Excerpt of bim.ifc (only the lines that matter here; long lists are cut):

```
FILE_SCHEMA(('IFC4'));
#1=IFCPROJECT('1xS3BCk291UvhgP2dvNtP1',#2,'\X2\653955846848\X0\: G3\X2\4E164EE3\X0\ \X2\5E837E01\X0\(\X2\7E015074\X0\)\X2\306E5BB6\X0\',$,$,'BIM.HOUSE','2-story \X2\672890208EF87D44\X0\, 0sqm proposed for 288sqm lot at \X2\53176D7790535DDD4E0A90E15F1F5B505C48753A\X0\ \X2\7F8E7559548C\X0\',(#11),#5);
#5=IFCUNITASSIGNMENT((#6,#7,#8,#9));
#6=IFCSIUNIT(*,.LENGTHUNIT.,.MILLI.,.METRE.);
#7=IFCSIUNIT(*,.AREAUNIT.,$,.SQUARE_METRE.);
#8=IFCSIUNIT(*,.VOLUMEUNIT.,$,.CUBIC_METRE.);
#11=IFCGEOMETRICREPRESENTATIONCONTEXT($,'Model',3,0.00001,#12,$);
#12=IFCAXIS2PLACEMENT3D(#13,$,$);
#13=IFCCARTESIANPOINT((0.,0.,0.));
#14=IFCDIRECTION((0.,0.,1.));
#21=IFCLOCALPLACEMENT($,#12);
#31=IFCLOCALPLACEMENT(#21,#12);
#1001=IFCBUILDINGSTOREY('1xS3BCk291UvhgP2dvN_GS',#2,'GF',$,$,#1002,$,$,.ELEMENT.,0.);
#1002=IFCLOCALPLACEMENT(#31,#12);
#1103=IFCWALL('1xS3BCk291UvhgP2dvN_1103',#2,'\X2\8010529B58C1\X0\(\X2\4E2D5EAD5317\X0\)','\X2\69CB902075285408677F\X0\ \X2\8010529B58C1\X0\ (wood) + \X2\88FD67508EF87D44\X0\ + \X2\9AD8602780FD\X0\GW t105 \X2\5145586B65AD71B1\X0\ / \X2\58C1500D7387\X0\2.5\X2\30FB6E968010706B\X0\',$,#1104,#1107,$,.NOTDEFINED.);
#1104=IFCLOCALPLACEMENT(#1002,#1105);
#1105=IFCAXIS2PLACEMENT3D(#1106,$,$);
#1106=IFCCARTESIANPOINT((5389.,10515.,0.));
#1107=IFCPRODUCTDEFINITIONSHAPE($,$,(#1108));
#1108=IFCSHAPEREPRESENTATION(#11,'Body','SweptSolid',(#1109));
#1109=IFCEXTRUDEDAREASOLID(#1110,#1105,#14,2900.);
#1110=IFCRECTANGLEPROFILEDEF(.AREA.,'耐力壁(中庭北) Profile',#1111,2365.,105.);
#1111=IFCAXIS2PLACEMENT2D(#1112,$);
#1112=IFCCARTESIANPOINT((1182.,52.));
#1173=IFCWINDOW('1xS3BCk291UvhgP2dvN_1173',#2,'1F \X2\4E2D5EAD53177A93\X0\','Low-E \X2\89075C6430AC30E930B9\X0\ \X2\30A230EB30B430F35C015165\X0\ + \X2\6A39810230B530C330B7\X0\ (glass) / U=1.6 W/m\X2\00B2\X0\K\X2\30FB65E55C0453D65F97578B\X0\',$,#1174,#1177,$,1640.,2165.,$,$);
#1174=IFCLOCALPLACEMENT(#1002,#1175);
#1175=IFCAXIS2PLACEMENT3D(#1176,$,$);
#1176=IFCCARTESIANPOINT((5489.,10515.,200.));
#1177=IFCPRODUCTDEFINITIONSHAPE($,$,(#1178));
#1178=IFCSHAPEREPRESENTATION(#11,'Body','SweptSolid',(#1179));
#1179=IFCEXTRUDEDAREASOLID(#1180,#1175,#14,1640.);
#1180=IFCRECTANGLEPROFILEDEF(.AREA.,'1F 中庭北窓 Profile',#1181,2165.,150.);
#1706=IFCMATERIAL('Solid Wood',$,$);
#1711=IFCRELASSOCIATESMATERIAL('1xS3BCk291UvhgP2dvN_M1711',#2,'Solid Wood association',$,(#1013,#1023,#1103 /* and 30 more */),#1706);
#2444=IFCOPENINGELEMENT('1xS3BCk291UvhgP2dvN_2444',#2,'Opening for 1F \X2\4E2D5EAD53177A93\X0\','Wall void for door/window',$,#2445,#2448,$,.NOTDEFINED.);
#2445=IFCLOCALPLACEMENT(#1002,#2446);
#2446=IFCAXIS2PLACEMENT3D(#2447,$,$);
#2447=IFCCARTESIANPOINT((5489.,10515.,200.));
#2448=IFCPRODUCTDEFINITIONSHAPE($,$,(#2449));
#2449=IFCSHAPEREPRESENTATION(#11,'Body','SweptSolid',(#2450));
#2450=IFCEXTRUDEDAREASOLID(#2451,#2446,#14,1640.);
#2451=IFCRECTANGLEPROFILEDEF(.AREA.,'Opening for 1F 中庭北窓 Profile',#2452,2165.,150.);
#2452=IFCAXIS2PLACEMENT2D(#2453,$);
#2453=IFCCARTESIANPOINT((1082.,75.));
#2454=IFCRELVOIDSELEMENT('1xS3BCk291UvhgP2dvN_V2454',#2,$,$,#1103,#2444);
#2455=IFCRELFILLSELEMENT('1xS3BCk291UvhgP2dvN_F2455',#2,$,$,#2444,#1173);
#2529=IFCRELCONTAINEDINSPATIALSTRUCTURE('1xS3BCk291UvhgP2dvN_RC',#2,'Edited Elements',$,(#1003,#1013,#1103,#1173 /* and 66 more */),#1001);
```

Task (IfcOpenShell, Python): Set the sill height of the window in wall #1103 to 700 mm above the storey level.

```python
import numpy as np
import ifcopenshell
import ifcopenshell.api.geometry
import ifcopenshell.geom
import ifcopenshell.util.element
import ifcopenshell.util.placement
import ifcopenshell.util.shape
import ifcopenshell.util.unit

model = ifcopenshell.open("bim.ifc")
unit_scale = ifcopenshell.util.unit.calculate_unit_scale(model)

window = model.by_guid("1xS3BCk291UvhgP2dvN_1173")
opening = window.FillsVoids[0].RelatingOpeningElement
storey = ifcopenshell.util.element.get_container(window, ifc_class="IfcBuildingStorey")
level = ifcopenshell.util.placement.get_local_placement(storey.ObjectPlacement)[2, 3]

# The opening's origin need not be at the sill, so measure its lowest point.
shape = ifcopenshell.geom.create_shape(ifcopenshell.geom.settings(), opening)
bottom = ifcopenshell.util.shape.get_shape_bottom_elevation(shape, shape.geometry) / unit_scale
dz = level + 700.0 - bottom

shift = np.array([0.0, 0.0, dz])
# The window is not placed relative to its opening, so move both.
for product in (opening, window):
    matrix = ifcopenshell.util.placement.get_local_placement(product.ObjectPlacement)
    matrix[:3, 3] += shift
    ifcopenshell.api.geometry.edit_object_placement(model, product=product, matrix=matrix, is_si=False)

print(f"moved by {dz * unit_scale:+.3f} m")

model.write("bim_rev.ifc")
```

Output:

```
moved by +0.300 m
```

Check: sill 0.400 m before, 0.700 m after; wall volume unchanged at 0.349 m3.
